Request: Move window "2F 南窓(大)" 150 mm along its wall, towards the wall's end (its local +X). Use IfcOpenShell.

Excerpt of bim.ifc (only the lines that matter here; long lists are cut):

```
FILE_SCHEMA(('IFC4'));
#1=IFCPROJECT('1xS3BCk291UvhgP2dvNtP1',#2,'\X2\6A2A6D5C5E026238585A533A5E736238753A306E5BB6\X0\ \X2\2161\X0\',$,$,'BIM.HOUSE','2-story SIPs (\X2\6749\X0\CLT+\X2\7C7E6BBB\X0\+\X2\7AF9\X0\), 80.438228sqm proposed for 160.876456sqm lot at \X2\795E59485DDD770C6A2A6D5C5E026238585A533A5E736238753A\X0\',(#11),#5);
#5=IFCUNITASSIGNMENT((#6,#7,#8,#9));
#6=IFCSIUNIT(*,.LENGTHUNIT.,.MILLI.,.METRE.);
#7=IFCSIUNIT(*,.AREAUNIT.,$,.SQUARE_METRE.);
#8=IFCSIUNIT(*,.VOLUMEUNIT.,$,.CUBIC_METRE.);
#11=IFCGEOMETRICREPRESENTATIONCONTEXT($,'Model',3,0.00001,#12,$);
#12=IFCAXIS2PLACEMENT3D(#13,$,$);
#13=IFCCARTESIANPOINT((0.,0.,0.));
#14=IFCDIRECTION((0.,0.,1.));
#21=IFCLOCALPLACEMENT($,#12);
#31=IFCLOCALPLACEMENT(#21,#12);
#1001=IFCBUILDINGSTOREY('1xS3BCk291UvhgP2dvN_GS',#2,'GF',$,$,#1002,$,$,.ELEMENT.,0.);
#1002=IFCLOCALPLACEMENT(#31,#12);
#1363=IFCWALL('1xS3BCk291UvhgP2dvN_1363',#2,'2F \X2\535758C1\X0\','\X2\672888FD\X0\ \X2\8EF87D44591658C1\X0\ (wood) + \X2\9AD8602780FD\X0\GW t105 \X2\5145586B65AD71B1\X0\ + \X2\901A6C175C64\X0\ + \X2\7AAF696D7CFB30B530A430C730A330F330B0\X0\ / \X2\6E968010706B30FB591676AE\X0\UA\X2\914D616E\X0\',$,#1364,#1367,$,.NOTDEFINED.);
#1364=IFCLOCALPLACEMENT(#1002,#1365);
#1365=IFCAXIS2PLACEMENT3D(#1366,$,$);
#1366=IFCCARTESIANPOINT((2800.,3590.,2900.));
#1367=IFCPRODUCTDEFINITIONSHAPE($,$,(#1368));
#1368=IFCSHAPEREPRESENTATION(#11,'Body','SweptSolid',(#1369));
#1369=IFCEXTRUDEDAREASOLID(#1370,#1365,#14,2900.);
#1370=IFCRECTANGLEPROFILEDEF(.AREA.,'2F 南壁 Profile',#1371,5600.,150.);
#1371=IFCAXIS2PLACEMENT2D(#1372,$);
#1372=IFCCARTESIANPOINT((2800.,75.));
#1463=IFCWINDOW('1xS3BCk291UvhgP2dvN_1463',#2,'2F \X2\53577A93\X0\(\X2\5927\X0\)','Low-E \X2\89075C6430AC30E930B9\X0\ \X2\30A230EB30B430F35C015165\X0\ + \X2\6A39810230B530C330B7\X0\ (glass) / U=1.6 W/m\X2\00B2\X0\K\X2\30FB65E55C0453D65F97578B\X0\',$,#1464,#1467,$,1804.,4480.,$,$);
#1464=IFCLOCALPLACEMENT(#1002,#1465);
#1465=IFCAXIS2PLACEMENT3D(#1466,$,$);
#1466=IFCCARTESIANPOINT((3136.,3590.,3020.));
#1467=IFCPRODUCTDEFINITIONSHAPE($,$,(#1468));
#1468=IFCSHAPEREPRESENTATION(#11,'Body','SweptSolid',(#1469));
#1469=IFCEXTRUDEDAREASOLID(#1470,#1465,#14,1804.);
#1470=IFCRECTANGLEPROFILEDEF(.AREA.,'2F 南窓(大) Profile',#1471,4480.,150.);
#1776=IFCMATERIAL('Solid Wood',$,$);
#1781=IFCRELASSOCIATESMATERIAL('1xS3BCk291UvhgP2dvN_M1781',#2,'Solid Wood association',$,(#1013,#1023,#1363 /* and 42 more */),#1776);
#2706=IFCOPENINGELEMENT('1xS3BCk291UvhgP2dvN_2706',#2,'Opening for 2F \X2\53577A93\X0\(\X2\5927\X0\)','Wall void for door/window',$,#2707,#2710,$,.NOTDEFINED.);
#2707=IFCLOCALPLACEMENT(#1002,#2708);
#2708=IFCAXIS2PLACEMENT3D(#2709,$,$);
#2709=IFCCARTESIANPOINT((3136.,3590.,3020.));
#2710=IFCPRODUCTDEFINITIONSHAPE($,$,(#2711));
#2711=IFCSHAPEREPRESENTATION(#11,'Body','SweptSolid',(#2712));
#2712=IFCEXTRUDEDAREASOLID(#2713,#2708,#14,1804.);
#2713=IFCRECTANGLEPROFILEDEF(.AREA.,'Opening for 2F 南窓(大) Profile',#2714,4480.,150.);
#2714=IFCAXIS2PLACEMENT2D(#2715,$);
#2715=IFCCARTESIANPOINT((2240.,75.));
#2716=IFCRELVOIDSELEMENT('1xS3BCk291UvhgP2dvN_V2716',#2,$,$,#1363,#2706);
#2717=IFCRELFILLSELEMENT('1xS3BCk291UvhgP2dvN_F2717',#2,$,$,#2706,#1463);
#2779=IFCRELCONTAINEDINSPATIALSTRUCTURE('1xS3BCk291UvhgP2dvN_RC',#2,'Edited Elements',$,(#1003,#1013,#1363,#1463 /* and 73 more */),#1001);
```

```python
import ifcopenshell
import ifcopenshell.api.geometry
import ifcopenshell.util.placement
import ifcopenshell.util.unit

model = ifcopenshell.open("bim.ifc")
unit_scale = ifcopenshell.util.unit.calculate_unit_scale(model)

window = model.by_id(1463)
opening = window.FillsVoids[0].RelatingOpeningElement
wall = opening.VoidsElements[0].RelatingBuildingElement

wall_matrix = ifcopenshell.util.placement.get_local_placement(wall.ObjectPlacement)
shift = wall_matrix[:3, 0] * 0.15 / unit_scale
before = ifcopenshell.util.placement.get_local_placement(window.ObjectPlacement)[:3, 3].copy()

# The window is not placed relative to its opening, so move both.
for product in (opening, window):
    matrix = ifcopenshell.util.placement.get_local_placement(product.ObjectPlacement)
    matrix[:3, 3] += shift
    ifcopenshell.api.geometry.edit_object_placement(model, product=product, matrix=matrix, is_si=False)

after = ifcopenshell.util.placement.get_local_placement(window.ObjectPlacement)[:3, 3]
print("window moved by", (after - before).round(3) + 0.0)

model.write("bim-out.ifc")
```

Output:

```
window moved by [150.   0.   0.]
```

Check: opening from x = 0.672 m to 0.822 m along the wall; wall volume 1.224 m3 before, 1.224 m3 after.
